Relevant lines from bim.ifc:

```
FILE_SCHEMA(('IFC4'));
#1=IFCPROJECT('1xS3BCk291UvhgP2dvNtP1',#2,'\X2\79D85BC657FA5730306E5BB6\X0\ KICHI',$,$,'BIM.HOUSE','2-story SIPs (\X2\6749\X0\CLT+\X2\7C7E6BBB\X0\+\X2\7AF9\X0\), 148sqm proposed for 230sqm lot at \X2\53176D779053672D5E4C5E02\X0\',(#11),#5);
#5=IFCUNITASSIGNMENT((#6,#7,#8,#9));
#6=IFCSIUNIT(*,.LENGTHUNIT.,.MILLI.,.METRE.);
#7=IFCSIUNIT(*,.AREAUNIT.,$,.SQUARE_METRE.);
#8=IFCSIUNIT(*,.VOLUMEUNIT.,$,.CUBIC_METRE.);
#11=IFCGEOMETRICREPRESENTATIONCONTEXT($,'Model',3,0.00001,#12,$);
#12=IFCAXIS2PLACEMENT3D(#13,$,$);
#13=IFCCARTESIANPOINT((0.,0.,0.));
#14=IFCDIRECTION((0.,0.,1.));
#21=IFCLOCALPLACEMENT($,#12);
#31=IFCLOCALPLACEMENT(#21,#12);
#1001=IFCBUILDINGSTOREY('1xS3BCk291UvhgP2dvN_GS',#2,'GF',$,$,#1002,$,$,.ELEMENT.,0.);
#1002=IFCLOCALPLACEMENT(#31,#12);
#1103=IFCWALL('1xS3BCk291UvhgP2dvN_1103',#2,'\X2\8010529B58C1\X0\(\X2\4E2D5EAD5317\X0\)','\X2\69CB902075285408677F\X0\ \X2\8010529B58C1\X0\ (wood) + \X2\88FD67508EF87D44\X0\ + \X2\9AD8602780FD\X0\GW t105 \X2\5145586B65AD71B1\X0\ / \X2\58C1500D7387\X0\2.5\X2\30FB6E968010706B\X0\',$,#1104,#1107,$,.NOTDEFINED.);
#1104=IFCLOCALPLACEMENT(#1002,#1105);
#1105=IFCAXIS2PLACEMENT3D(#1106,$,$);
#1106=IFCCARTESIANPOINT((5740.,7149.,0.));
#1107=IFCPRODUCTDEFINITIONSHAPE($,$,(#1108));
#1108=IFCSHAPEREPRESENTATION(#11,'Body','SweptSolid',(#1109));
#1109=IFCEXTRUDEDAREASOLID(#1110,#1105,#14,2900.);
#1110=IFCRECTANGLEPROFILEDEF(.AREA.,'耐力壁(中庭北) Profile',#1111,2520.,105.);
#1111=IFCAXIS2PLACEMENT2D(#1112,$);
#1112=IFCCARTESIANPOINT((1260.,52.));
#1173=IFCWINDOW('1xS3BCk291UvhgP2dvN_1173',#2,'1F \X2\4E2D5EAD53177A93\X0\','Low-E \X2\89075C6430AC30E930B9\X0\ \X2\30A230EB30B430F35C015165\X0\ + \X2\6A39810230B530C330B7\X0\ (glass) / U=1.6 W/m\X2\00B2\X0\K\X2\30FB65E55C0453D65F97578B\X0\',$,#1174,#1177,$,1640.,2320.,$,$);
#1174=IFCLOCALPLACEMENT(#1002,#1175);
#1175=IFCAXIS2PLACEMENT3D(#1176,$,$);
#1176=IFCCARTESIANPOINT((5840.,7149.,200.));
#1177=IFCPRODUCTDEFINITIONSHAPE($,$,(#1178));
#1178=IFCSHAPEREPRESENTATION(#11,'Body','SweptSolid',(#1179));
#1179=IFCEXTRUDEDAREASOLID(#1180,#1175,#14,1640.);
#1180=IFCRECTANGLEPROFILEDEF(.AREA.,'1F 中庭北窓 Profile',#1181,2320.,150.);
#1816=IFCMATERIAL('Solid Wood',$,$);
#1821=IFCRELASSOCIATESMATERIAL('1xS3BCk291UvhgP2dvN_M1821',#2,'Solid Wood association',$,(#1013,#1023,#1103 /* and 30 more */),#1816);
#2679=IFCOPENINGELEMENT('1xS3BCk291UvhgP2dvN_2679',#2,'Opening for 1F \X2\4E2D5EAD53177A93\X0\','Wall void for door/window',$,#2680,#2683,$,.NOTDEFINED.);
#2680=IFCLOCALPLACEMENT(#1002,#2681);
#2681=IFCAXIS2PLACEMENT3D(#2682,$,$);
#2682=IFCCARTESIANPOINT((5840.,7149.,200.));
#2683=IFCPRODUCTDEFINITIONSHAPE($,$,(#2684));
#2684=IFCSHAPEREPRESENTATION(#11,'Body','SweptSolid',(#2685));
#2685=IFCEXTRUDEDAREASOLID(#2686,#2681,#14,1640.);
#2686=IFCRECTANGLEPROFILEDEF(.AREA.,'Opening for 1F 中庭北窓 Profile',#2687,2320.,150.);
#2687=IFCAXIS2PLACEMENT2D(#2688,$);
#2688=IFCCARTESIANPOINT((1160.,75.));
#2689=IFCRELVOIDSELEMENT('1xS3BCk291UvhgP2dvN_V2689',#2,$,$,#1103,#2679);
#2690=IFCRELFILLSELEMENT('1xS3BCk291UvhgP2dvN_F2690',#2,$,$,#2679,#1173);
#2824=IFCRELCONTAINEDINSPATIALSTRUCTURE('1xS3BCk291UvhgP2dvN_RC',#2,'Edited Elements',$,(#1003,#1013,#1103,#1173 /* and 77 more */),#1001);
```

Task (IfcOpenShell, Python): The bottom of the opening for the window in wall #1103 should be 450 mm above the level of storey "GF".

```python
import numpy as np
import ifcopenshell
import ifcopenshell.api.geometry
import ifcopenshell.geom
import ifcopenshell.util.element
import ifcopenshell.util.placement
import ifcopenshell.util.shape
import ifcopenshell.util.unit

model = ifcopenshell.open("bim.ifc")
unit_scale = ifcopenshell.util.unit.calculate_unit_scale(model)

window = model.by_guid("1xS3BCk291UvhgP2dvN_1173")
opening = window.FillsVoids[0].RelatingOpeningElement
storey = ifcopenshell.util.element.get_container(window, ifc_class="IfcBuildingStorey")
level = ifcopenshell.util.placement.get_local_placement(storey.ObjectPlacement)[2, 3]

# The opening's origin need not be at the sill, so measure its lowest point.
shape = ifcopenshell.geom.create_shape(ifcopenshell.geom.settings(), opening)
bottom = ifcopenshell.util.shape.get_shape_bottom_elevation(shape, shape.geometry) / unit_scale
dz = level + 450.0 - bottom

shift = np.array([0.0, 0.0, dz])
# The window is not placed relative to its opening, so move both.
for product in (opening, window):
    matrix = ifcopenshell.util.placement.get_local_placement(product.ObjectPlacement)
    matrix[:3, 3] += shift
    ifcopenshell.api.geometry.edit_object_placement(model, product=product, matrix=matrix, is_si=False)

print(f"moved by {dz * unit_scale:+.3f} m")

model.write("bim-out.ifc")
```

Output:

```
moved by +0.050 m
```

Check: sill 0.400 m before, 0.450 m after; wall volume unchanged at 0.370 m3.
